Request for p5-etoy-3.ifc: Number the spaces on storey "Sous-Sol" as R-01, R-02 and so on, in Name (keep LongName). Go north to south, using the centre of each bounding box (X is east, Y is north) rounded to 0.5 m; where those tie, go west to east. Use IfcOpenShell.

First a look at what the model holds.

```python
import ifcopenshell
import ifcopenshell.util.element
import ifcopenshell.util.placement

model = ifcopenshell.open("p5-etoy-3.ifc")
print(model.schema)
storey = next(s for s in model.by_type("IfcBuildingStorey") if s.Name == "Sous-Sol")
spaces = [e for e in ifcopenshell.util.element.get_decomposition(storey) if e.is_a("IfcSpace")]
for e in sorted(spaces, key=lambda e: e.id()):
    origin = ifcopenshell.util.placement.get_local_placement(e.ObjectPlacement)[:3, 3]
    print(e.id(), e.Name, e.LongName, origin.round(2) + 0.0, sep=" | ")
```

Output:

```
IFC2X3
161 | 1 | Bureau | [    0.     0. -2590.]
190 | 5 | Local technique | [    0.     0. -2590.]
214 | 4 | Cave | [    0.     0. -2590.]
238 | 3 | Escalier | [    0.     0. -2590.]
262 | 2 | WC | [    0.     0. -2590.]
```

```python
import ifcopenshell
import ifcopenshell.geom
import ifcopenshell.util.element
import ifcopenshell.util.shape

model = ifcopenshell.open("p5-etoy-3.ifc")
settings = ifcopenshell.geom.settings()
settings.set("use-world-coords", True)


def centre(element):
    shape = ifcopenshell.geom.create_shape(settings, element)
    return ifcopenshell.util.shape.get_bbox_centroid(shape.geometry)


storey = next(s for s in model.by_type("IfcBuildingStorey") if s.Name == "Sous-Sol")
spaces = [e for e in ifcopenshell.util.element.get_decomposition(storey) if e.is_a("IfcSpace")]

# Insertion points can sit at a corner or the storey origin, so sort by the geometry (in metres).
centres = {e: centre(e) for e in spaces}
spaces.sort(key=lambda e: (-round(centres[e][1] / 0.5), centres[e][0]))

for i, e in enumerate(spaces, start=1):
    number = f"R-{i:02d}"
    e.Name = number
    print(e.id(), number)

model.write("p5-etoy-3_v2.ifc")
```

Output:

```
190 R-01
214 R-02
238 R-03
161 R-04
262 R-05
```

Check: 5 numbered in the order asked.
